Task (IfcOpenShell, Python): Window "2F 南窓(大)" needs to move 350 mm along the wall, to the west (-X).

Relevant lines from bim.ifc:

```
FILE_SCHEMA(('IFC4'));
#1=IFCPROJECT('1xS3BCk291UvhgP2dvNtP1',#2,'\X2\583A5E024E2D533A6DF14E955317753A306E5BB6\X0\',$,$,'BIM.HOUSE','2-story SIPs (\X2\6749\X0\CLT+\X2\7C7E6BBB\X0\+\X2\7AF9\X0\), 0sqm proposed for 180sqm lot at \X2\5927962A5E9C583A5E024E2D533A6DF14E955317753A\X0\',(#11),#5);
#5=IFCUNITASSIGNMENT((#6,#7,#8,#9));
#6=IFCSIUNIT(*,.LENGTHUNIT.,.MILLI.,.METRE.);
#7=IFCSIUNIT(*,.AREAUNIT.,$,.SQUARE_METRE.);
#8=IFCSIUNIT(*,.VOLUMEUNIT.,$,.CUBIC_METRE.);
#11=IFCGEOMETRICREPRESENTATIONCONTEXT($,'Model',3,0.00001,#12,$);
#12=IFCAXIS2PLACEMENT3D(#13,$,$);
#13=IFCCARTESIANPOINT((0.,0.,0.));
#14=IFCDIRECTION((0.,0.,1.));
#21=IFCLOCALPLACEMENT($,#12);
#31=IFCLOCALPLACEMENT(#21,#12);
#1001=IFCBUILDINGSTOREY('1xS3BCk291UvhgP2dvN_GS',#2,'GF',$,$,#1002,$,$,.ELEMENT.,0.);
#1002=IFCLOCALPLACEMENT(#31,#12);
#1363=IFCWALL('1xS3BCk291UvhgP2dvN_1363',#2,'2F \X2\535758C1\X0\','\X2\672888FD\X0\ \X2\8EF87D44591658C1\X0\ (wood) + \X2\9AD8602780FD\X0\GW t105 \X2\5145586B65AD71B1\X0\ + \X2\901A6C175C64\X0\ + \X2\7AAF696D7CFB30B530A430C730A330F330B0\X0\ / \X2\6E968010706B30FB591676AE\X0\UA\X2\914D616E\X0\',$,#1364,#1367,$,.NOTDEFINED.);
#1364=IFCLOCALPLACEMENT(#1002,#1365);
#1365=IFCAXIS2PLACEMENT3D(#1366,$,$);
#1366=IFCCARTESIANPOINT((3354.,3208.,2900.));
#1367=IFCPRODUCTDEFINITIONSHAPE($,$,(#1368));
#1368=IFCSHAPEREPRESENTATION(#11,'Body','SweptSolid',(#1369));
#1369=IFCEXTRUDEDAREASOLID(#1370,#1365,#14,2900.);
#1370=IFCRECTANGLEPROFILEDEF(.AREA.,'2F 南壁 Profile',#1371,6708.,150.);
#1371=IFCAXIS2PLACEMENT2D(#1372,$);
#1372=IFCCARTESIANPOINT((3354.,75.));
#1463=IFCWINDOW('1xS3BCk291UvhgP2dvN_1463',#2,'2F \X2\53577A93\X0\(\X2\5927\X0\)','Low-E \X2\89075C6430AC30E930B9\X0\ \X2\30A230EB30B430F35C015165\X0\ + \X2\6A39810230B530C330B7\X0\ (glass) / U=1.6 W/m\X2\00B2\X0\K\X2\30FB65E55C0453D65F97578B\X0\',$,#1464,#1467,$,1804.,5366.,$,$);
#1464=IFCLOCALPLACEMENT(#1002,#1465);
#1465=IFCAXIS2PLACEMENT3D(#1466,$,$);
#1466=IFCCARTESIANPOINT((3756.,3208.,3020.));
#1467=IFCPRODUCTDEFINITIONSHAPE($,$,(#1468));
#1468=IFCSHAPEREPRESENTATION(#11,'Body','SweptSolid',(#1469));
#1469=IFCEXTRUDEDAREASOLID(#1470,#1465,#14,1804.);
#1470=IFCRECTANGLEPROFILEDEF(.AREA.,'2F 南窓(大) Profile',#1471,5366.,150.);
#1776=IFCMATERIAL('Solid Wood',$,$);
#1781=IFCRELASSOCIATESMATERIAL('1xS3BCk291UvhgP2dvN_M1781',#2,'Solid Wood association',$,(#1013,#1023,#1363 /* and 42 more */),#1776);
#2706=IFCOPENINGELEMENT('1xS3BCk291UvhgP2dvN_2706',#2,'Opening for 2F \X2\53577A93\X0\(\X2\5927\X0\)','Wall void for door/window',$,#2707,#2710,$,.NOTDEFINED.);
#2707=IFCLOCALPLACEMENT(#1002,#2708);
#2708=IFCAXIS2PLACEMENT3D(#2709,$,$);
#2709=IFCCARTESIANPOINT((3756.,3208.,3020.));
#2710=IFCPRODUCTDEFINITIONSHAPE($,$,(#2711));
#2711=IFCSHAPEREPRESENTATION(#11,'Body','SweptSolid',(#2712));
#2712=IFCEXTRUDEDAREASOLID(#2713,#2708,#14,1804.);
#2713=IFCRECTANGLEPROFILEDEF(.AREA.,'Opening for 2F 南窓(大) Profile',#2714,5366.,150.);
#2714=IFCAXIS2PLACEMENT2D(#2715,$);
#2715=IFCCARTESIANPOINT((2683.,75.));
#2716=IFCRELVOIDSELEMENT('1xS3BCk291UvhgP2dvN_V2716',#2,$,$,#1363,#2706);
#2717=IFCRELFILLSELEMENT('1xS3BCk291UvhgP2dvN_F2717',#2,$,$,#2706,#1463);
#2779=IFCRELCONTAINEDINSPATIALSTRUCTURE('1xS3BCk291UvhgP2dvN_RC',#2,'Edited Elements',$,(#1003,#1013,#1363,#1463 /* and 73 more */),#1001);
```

```python
import ifcopenshell
import ifcopenshell.api.geometry
import ifcopenshell.util.placement

model = ifcopenshell.open("bim.ifc")

window = model.by_guid("1xS3BCk291UvhgP2dvN_1463")
opening = window.FillsVoids[0].RelatingOpeningElement
wall = opening.VoidsElements[0].RelatingBuildingElement

wall_matrix = ifcopenshell.util.placement.get_local_placement(wall.ObjectPlacement)
shift = wall_matrix[:3, 0] * -350.0
before = ifcopenshell.util.placement.get_local_placement(window.ObjectPlacement)[:3, 3].copy()

# The window is not placed relative to its opening, so move both.
for product in (opening, window):
    matrix = ifcopenshell.util.placement.get_local_placement(product.ObjectPlacement)
    matrix[:3, 3] += shift
    ifcopenshell.api.geometry.edit_object_placement(model, product=product, matrix=matrix, is_si=False)

after = ifcopenshell.util.placement.get_local_placement(window.ObjectPlacement)[:3, 3]
print("window moved by", (after - before).round(3) + 0.0)

model.write("bim_updated.ifc")
```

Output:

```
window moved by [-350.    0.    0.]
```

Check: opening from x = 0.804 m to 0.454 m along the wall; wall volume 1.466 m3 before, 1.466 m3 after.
